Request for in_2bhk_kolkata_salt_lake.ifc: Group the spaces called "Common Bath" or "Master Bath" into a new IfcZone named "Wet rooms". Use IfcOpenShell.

First a look at what the model holds.

```python
import ifcopenshell

model = ifcopenshell.open("in_2bhk_kolkata_salt_lake.ifc")
print(model.schema)
seen = {}
for space in model.by_type("IfcSpace"):
    seen[space.LongName] = seen.get(space.LongName, 0) + 1
for name, count in sorted(seen.items(), key=str):
    print(count, "x", name)
print("zones:", [z.Name for z in model.by_type("IfcZone")][:20])
```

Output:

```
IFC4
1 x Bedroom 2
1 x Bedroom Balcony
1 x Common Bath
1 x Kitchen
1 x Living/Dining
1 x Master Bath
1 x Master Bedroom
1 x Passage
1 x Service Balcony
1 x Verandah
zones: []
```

```python
import ifcopenshell
import ifcopenshell.api.group
import ifcopenshell.api.root

model = ifcopenshell.open("in_2bhk_kolkata_salt_lake.ifc")

names = {"Common Bath", "Master Bath"}
spaces = [s for s in model.by_type("IfcSpace") if s.LongName in names]

zone = ifcopenshell.api.root.create_entity(model, ifc_class="IfcZone", name="Wet rooms")
ifcopenshell.api.group.assign_group(model, products=spaces, group=zone)
print(len(spaces), "spaces in", zone.Name)

model.write("in_2bhk_kolkata_salt_lake_rev.ifc")
```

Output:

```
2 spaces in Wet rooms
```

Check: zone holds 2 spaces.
